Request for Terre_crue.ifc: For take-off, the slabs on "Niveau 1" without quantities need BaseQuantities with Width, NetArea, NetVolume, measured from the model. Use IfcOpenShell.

First a look at what the model holds.

```python
import ifcopenshell
import ifcopenshell.util.element
import ifcopenshell.util.unit

model = ifcopenshell.open("Terre_crue.ifc")
print(model.schema)
for unit_type in ("LENGTHUNIT", "AREAUNIT", "VOLUMEUNIT"):
    print(unit_type, ifcopenshell.util.unit.calculate_unit_scale(model, unit_type))
storey = next(s for s in model.by_type("IfcBuildingStorey") if s.Name == "Niveau 1")
slabs = [e for e in ifcopenshell.util.element.get_decomposition(storey) if e.is_a("IfcSlab")]
for e in sorted(slabs, key=lambda e: e.id()):
    print(e.id(), e.is_a(), e.Name, list(ifcopenshell.util.element.get_psets(e, qtos_only=True)), sep=" | ")
```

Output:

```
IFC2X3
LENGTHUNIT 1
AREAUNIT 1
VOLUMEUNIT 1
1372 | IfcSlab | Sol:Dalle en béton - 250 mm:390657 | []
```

```python
import ifcopenshell
import ifcopenshell.api.pset
import ifcopenshell.geom
import ifcopenshell.util.element
import ifcopenshell.util.shape
import ifcopenshell.util.unit

model = ifcopenshell.open("Terre_crue.ifc")
unit_scale = ifcopenshell.util.unit.calculate_unit_scale(model)
area_scale = ifcopenshell.util.unit.calculate_unit_scale(model, "AREAUNIT")
volume_scale = ifcopenshell.util.unit.calculate_unit_scale(model, "VOLUMEUNIT")
settings = ifcopenshell.geom.settings()

storey = next(s for s in model.by_type("IfcBuildingStorey") if s.Name == "Niveau 1")
slabs = [e for e in ifcopenshell.util.element.get_decomposition(storey) if e.is_a("IfcSlab")]

for e in sorted(slabs, key=lambda e: e.id()):
    if ifcopenshell.util.element.get_psets(e, qtos_only=True, should_inherit=False):
        continue
    # Geometry comes back in metres, in the element's own axes.
    shape = ifcopenshell.geom.create_shape(settings, e)
    values = {
        "Width": ifcopenshell.util.shape.get_z(shape.geometry) / unit_scale,
        "NetArea": ifcopenshell.util.shape.get_footprint_area(shape.geometry) / area_scale,
        "NetVolume": ifcopenshell.util.shape.get_volume(shape.geometry) / volume_scale,
    }
    qto = ifcopenshell.api.pset.add_qto(model, product=e, name="BaseQuantities")
    ifcopenshell.api.pset.edit_qto(model, qto=qto, properties=values)
    print(e.id(), {k: round(v, 3) for k, v in values.items()})

model.write("Terre_crue-out.ifc")
```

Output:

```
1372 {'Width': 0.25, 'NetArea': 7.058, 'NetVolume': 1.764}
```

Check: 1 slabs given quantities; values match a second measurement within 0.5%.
